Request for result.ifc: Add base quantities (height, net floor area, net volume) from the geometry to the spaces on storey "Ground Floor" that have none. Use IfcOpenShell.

First a look at what the model holds.

```python
import ifcopenshell
import ifcopenshell.util.element
import ifcopenshell.util.unit

model = ifcopenshell.open("result.ifc")
print(model.schema)
for unit_type in ("LENGTHUNIT", "AREAUNIT", "VOLUMEUNIT"):
    print(unit_type, ifcopenshell.util.unit.calculate_unit_scale(model, unit_type))
storey = next(s for s in model.by_type("IfcBuildingStorey") if s.Name == "Ground Floor")
spaces = [e for e in ifcopenshell.util.element.get_decomposition(storey) if e.is_a("IfcSpace")]
for e in sorted(spaces, key=lambda e: e.id()):
    print(e.id(), e.is_a(), e.Name, list(ifcopenshell.util.element.get_psets(e, qtos_only=True)), sep=" | ")
```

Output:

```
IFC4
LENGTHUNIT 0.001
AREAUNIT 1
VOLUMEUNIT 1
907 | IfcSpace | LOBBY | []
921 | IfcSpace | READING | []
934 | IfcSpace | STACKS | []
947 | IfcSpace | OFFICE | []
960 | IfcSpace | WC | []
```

```python
import ifcopenshell
import ifcopenshell.api.pset
import ifcopenshell.geom
import ifcopenshell.util.element
import ifcopenshell.util.shape
import ifcopenshell.util.unit

model = ifcopenshell.open("result.ifc")
unit_scale = ifcopenshell.util.unit.calculate_unit_scale(model)
area_scale = ifcopenshell.util.unit.calculate_unit_scale(model, "AREAUNIT")
volume_scale = ifcopenshell.util.unit.calculate_unit_scale(model, "VOLUMEUNIT")
settings = ifcopenshell.geom.settings()

storey = next(s for s in model.by_type("IfcBuildingStorey") if s.Name == "Ground Floor")
spaces = [e for e in ifcopenshell.util.element.get_decomposition(storey) if e.is_a("IfcSpace")]

for e in sorted(spaces, key=lambda e: e.id()):
    if ifcopenshell.util.element.get_psets(e, qtos_only=True, should_inherit=False):
        continue
    # Geometry comes back in metres, in the element's own axes.
    shape = ifcopenshell.geom.create_shape(settings, e)
    values = {
        "Height": ifcopenshell.util.shape.get_z(shape.geometry) / unit_scale,
        "NetFloorArea": ifcopenshell.util.shape.get_footprint_area(shape.geometry) / area_scale,
        "NetVolume": ifcopenshell.util.shape.get_volume(shape.geometry) / volume_scale,
    }
    qto = ifcopenshell.api.pset.add_qto(model, product=e, name="Qto_SpaceBaseQuantities")
    ifcopenshell.api.pset.edit_qto(model, qto=qto, properties=values)
    print(e.id(), {k: round(v, 3) for k, v in values.items()})

model.write("result-out.ifc")
```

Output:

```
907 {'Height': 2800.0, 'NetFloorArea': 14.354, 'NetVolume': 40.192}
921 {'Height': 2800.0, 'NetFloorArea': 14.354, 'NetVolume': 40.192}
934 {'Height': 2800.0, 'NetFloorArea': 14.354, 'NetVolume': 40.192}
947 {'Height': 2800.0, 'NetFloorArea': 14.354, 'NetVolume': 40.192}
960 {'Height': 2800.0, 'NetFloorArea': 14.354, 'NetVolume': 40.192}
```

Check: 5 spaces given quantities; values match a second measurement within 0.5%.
